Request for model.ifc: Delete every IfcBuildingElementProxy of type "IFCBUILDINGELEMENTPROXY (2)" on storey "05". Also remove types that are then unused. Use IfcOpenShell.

First a look at what the model holds.

```python
import ifcopenshell
import ifcopenshell.util.element

model = ifcopenshell.open("model.ifc")
print(model.schema)
storey = next(s for s in model.by_type("IfcBuildingStorey") if s.Name == "05")
proxies = [e for e in ifcopenshell.util.element.get_decomposition(storey) if e.is_a("IfcBuildingElementProxy")]
seen = {}
for e in proxies:
    element_type = ifcopenshell.util.element.get_type(e)
    name = element_type.Name if element_type not in (None, e) else None
    seen[name] = seen.get(name, 0) + 1
for name, count in sorted(seen.items(), key=str):
    print(count, "x", name)
```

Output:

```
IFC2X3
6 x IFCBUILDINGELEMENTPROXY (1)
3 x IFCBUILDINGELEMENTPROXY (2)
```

```python
import ifcopenshell
import ifcopenshell.api.root
import ifcopenshell.util.element

model = ifcopenshell.open("model.ifc")

storey = next(s for s in model.by_type("IfcBuildingStorey") if s.Name == "05")
proxies = [e for e in ifcopenshell.util.element.get_decomposition(storey) if e.is_a("IfcBuildingElementProxy")]
targets = [e for e in proxies if (t := ifcopenshell.util.element.get_type(e)) not in (None, e) and t.Name == "IFCBUILDINGELEMENTPROXY (2)"]
types = {ifcopenshell.util.element.get_type(e) for e in targets} - {None, *targets}

for e in targets:
    ifcopenshell.api.root.remove_product(model, product=e)
print(len(targets), "removed")

unused = [t for t in types if not ifcopenshell.util.element.get_types(t)]
for t in unused:
    ifcopenshell.api.root.remove_product(model, product=t)
print(len(unused), "unused types removed")

model.write("model_updated.ifc")
```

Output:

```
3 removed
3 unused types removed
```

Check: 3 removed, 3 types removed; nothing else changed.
